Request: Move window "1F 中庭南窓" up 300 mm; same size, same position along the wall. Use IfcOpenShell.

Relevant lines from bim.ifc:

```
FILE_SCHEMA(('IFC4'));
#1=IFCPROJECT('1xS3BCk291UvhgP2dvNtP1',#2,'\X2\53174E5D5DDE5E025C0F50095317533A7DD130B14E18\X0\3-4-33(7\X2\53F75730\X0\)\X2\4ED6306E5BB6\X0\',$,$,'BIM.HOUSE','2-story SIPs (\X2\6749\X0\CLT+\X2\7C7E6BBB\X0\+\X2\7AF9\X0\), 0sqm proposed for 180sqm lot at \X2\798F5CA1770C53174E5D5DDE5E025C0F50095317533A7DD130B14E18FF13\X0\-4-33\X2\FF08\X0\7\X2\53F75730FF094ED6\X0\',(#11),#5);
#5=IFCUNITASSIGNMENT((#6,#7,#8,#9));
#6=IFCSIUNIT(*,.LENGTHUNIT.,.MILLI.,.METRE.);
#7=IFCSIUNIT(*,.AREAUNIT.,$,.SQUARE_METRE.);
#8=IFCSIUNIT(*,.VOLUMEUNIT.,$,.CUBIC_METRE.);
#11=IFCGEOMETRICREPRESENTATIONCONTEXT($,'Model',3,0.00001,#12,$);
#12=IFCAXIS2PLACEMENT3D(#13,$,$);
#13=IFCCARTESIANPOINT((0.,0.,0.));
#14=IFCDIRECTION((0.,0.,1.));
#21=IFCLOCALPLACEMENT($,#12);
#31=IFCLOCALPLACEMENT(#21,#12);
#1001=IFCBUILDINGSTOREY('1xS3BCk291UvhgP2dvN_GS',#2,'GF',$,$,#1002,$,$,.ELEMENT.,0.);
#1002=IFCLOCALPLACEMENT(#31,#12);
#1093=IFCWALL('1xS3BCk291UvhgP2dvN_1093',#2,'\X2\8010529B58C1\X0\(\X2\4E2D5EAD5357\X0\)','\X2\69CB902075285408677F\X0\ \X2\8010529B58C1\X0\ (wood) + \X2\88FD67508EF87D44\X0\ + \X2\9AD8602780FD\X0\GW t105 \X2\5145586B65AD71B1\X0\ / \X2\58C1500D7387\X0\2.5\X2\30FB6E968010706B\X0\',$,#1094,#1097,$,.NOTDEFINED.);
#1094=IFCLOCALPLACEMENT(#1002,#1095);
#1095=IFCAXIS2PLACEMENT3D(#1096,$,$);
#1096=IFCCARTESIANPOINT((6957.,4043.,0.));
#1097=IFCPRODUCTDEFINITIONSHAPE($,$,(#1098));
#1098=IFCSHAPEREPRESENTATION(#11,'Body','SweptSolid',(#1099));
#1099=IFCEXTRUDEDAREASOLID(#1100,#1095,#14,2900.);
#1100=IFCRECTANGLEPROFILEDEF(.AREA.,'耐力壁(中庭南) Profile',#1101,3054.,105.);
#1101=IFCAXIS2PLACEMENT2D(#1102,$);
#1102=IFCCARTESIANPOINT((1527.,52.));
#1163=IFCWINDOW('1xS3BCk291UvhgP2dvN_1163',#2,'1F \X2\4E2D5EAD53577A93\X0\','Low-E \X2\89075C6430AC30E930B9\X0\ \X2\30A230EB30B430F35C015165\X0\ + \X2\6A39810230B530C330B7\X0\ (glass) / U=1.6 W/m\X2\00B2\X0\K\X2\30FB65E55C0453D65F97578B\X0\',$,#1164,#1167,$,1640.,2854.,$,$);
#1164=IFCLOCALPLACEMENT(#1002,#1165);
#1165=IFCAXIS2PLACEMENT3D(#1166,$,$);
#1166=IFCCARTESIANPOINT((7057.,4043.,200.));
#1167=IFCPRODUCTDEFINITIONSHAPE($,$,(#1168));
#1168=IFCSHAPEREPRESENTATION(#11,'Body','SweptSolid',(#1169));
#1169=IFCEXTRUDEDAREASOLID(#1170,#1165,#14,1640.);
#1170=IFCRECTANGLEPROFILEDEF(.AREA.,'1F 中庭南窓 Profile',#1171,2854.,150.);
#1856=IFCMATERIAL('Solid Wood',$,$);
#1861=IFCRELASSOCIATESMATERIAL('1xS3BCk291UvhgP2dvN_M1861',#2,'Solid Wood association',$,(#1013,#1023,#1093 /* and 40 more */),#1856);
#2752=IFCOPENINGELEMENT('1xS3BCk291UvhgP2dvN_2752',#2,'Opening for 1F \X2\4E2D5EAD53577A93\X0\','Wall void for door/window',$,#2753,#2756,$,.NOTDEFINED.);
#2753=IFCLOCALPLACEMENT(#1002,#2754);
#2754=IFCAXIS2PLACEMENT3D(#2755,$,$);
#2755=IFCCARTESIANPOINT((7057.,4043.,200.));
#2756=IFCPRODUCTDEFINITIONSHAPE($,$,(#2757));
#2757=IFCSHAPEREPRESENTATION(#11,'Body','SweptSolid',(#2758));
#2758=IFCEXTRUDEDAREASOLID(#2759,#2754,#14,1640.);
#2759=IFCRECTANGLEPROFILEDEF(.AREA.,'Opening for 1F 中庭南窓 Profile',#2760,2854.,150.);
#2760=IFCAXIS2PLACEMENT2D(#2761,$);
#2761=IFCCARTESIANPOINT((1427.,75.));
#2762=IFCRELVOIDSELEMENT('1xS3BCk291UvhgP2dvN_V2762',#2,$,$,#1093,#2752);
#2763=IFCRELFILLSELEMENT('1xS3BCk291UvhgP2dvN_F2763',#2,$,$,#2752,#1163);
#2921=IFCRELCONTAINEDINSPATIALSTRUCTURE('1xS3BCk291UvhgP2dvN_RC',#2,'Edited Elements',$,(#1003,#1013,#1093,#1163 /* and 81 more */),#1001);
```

```python
import numpy as np
import ifcopenshell
import ifcopenshell.api.geometry
import ifcopenshell.util.placement
import ifcopenshell.util.unit

model = ifcopenshell.open("bim.ifc")
unit_scale = ifcopenshell.util.unit.calculate_unit_scale(model)

window = model.by_guid("1xS3BCk291UvhgP2dvN_1163")
opening = window.FillsVoids[0].RelatingOpeningElement
dz = 0.3 / unit_scale

shift = np.array([0.0, 0.0, dz])
# The window is not placed relative to its opening, so move both.
for product in (opening, window):
    matrix = ifcopenshell.util.placement.get_local_placement(product.ObjectPlacement)
    matrix[:3, 3] += shift
    ifcopenshell.api.geometry.edit_object_placement(model, product=product, matrix=matrix, is_si=False)

print(f"moved by {dz * unit_scale:+.3f} m")

model.write("bim_edited.ifc")
```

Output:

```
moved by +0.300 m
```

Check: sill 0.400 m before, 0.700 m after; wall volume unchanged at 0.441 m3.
